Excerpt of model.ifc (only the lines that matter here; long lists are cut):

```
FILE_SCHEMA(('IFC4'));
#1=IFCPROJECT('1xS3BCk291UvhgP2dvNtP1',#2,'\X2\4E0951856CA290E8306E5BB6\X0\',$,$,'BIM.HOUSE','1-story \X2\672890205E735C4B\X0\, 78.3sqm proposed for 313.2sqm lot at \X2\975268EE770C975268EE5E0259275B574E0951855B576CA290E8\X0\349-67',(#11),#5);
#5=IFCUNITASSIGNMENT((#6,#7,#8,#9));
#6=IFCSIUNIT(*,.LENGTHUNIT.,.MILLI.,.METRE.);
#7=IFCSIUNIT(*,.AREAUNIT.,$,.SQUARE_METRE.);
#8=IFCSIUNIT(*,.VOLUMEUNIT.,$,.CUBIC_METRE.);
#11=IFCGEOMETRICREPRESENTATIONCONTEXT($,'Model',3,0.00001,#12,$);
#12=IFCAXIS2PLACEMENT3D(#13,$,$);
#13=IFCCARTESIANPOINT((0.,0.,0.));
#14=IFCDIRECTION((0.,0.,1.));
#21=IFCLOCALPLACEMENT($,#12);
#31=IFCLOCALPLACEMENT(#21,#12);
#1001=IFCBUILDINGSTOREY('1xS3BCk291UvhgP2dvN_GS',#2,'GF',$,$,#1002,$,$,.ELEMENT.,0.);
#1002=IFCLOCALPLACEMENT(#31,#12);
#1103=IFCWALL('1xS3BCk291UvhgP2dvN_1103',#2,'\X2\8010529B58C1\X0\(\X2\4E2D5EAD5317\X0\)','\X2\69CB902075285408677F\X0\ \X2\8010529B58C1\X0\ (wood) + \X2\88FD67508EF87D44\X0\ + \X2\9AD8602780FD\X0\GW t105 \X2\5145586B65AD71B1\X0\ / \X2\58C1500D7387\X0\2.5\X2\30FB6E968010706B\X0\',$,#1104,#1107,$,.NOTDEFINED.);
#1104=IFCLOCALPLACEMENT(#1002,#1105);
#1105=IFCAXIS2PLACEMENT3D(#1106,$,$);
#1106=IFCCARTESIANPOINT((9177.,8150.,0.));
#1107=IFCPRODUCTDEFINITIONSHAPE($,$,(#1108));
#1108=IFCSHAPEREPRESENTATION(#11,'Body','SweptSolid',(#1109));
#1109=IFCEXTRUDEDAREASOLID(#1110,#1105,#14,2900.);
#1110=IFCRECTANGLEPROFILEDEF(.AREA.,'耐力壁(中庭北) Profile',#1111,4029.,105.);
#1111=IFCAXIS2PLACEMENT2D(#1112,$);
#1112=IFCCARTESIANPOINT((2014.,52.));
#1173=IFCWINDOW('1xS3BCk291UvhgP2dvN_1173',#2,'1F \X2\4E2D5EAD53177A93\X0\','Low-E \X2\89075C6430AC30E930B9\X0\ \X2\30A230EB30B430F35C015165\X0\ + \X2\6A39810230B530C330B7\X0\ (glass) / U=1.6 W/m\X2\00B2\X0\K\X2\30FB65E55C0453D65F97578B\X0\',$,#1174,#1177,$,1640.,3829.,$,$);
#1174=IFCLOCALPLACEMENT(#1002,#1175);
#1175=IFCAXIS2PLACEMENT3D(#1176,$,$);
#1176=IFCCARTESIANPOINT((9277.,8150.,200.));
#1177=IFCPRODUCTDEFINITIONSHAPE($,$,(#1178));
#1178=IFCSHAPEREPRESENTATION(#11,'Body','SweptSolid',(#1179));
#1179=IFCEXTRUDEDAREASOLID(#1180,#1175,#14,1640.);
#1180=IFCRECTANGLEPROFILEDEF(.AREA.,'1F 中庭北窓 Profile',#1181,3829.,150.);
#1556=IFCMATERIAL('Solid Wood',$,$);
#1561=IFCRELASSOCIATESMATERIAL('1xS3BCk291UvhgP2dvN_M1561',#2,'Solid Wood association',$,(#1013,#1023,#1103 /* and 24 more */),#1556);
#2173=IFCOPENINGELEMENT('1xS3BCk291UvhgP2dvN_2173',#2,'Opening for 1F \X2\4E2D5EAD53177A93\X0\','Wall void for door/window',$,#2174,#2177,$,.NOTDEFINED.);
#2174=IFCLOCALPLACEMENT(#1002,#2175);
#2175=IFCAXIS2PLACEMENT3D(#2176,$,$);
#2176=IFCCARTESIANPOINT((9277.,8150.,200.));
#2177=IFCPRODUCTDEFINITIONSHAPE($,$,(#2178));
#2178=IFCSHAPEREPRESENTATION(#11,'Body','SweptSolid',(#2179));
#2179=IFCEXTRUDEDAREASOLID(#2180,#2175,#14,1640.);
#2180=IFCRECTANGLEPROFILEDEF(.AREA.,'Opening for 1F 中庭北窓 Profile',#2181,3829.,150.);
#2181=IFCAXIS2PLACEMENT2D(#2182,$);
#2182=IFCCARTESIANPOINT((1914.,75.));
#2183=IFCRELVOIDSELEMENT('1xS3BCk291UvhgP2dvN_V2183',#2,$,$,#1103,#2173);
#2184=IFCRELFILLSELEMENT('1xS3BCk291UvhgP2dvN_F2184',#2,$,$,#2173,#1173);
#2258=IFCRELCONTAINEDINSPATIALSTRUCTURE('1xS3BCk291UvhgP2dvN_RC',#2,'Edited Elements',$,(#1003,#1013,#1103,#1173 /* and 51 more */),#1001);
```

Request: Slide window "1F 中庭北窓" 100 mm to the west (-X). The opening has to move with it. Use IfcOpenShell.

```python
import ifcopenshell
import ifcopenshell.api.geometry
import ifcopenshell.util.placement
import ifcopenshell.util.unit

model = ifcopenshell.open("model.ifc")
unit_scale = ifcopenshell.util.unit.calculate_unit_scale(model)

window = model.by_guid("1xS3BCk291UvhgP2dvN_1173")
opening = window.FillsVoids[0].RelatingOpeningElement
wall = opening.VoidsElements[0].RelatingBuildingElement

wall_matrix = ifcopenshell.util.placement.get_local_placement(wall.ObjectPlacement)
shift = wall_matrix[:3, 0] * -0.1 / unit_scale
before = ifcopenshell.util.placement.get_local_placement(window.ObjectPlacement)[:3, 3].copy()

# The window is not placed relative to its opening, so move both.
for product in (opening, window):
    matrix = ifcopenshell.util.placement.get_local_placement(product.ObjectPlacement)
    matrix[:3, 3] += shift
    ifcopenshell.api.geometry.edit_object_placement(model, product=product, matrix=matrix, is_si=False)

after = ifcopenshell.util.placement.get_local_placement(window.ObjectPlacement)[:3, 3]
print("window moved by", (after - before).round(3) + 0.0)

model.write("model_updated.ifc")
```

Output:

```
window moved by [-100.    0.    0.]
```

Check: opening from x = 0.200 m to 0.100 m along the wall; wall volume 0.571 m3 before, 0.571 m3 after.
